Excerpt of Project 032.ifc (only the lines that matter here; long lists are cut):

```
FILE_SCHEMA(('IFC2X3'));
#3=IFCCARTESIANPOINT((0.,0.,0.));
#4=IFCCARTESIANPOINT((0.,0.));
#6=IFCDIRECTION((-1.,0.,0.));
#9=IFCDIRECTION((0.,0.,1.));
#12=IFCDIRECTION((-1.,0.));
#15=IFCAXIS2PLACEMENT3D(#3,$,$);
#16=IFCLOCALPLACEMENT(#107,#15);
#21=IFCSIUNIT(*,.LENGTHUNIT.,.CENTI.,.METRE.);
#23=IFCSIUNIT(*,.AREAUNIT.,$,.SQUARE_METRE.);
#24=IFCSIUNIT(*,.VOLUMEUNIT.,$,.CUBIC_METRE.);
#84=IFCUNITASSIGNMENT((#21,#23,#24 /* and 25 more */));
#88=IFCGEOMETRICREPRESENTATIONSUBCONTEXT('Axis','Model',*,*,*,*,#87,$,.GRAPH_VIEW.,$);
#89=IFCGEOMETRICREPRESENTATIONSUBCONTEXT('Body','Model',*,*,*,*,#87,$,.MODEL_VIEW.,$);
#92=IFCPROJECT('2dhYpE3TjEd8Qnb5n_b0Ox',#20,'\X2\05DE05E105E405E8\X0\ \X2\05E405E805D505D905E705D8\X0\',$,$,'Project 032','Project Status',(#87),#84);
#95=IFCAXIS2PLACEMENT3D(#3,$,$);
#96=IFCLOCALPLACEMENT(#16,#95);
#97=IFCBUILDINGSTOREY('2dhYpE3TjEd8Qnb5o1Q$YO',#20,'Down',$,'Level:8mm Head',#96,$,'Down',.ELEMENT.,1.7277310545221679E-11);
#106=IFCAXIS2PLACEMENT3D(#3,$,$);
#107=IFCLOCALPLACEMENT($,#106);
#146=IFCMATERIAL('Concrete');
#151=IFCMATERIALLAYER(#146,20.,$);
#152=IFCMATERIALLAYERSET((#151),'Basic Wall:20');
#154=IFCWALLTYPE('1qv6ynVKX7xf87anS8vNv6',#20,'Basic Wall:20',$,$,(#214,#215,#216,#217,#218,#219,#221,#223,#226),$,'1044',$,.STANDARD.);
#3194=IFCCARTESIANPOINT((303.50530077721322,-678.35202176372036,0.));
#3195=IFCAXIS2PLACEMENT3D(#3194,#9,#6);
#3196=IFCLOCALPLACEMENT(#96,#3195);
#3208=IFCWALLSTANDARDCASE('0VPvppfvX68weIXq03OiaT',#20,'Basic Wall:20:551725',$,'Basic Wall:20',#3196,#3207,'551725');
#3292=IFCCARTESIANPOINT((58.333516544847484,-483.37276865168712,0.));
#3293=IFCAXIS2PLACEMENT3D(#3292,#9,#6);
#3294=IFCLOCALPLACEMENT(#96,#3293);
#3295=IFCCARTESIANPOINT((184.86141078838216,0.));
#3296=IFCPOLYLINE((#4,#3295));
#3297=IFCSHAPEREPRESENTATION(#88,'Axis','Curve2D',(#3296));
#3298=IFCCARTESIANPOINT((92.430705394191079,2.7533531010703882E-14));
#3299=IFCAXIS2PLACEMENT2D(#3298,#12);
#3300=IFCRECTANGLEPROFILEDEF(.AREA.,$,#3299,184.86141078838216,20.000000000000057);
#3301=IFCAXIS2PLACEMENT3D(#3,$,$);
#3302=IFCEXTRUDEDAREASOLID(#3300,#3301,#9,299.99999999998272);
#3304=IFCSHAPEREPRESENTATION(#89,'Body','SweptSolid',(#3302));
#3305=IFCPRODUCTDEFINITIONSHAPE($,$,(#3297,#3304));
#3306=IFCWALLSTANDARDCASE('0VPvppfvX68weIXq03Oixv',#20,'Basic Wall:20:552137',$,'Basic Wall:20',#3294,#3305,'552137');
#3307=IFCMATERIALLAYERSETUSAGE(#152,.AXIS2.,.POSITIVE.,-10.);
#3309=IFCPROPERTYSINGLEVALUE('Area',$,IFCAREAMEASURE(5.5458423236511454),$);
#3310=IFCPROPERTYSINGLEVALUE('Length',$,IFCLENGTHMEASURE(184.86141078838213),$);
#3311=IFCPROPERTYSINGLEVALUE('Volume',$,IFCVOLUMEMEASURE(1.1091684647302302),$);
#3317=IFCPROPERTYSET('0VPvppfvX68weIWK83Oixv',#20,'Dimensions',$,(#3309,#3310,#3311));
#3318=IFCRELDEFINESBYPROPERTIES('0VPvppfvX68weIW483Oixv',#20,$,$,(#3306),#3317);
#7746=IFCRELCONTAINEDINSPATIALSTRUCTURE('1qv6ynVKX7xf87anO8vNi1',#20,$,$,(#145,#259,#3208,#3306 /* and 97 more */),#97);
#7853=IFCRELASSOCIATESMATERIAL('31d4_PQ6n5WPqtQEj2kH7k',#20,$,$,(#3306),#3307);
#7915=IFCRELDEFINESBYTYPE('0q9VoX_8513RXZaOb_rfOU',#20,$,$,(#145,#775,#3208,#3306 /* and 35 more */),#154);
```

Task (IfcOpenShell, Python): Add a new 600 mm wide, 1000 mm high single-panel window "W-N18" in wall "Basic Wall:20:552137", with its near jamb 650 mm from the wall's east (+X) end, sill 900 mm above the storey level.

```python
import numpy as np
import ifcopenshell
import ifcopenshell.api.feature
import ifcopenshell.api.geometry
import ifcopenshell.api.pset
import ifcopenshell.api.root
import ifcopenshell.api.spatial
import ifcopenshell.api.type
import ifcopenshell.geom
import ifcopenshell.util.element
import ifcopenshell.util.placement
import ifcopenshell.util.representation
import ifcopenshell.util.shape
import ifcopenshell.util.unit

model = ifcopenshell.open("Project 032.ifc")
unit_scale = ifcopenshell.util.unit.calculate_unit_scale(model)
area_scale = ifcopenshell.util.unit.calculate_unit_scale(model, "AREAUNIT")
volume_scale = ifcopenshell.util.unit.calculate_unit_scale(model, "VOLUMEUNIT")
settings = ifcopenshell.geom.settings()


def volume(element):
    """Net volume in cubic metres, openings subtracted."""
    shape = ifcopenshell.geom.create_shape(settings, element)
    return ifcopenshell.util.shape.get_volume(shape.geometry)


wall = model.by_guid("0VPvppfvX68weIXq03Oixv")
storey = ifcopenshell.util.element.get_container(wall, ifc_class="IfcBuildingStorey")
context = ifcopenshell.util.representation.get_context(model, "Model", "Body", "MODEL_VIEW")
before = volume(wall)

width, height, from_end, sill = 0.6, 1, 0.65, 0.9  # metres

# The wall runs along its own X axis, and the end named is its -X end.
wall_shape = ifcopenshell.geom.create_shape(settings, wall)
x, y, z = ifcopenshell.util.shape.get_vertices(wall_shape.geometry).T
start = x.min() + from_end
face, thickness = float(y.min()), float(y.max() - y.min())
wall_matrix = ifcopenshell.util.placement.get_local_placement(wall.ObjectPlacement)
level = ifcopenshell.util.placement.get_local_placement(storey.ObjectPlacement)[2, 3]


def in_wall(x, y):
    """Placement at x, y metres in the wall's axes, at sill height."""
    matrix = wall_matrix.copy()
    matrix[:, 3] = wall_matrix @ np.array([x / unit_scale, y / unit_scale, 0.0, 1.0])
    matrix[2, 3] = level + sill / unit_scale
    return matrix


# Opening: a box that overshoots both wall faces by 50 mm.
opening = ifcopenshell.api.root.create_entity(model, ifc_class="IfcOpeningElement")
box = ifcopenshell.api.geometry.add_wall_representation(
    model, context=context, length=width, height=height, thickness=thickness + 0.1
)
ifcopenshell.api.geometry.assign_representation(model, product=opening, representation=box)
ifcopenshell.api.geometry.edit_object_placement(model, product=opening, matrix=in_wall(start, face - 0.05), is_si=False)
ifcopenshell.api.feature.add_feature(model, feature=opening, element=wall)

window = ifcopenshell.api.root.create_entity(model, ifc_class="IfcWindow", name="W-N18")
window.OverallWidth, window.OverallHeight = width / unit_scale, height / unit_scale
body = ifcopenshell.api.geometry.add_window_representation(
    model,
    context=context,
    overall_width=window.OverallWidth,
    overall_height=window.OverallHeight,
    partition_type="SINGLE_PANEL",
)
ifcopenshell.api.geometry.assign_representation(model, product=window, representation=body)
ifcopenshell.api.spatial.assign_container(model, products=[window], relating_structure=storey)
fills = ifcopenshell.api.feature.add_filling(model, opening=opening, element=window)
fills.OwnerHistory = window.OwnerHistory  # required in IFC2X3

# IFC2X3 keeps the operation on the window style.
style = ifcopenshell.api.root.create_entity(model, ifc_class="IfcWindowStyle", name="W-N18")
style.OperationType, style.ConstructionType = "SINGLE_PANEL", "NOTDEFINED"
style.ParameterTakesPrecedence = style.Sizeable = False
ifcopenshell.api.type.assign_type(model, related_objects=[window], relating_type=style)

# Centre the window in the wall's thickness.
ifcopenshell.api.geometry.edit_object_placement(model, product=window, matrix=in_wall(start, face), is_si=False)
window_shape = ifcopenshell.geom.create_shape(settings, window)
depth = ifcopenshell.util.shape.get_vertices(window_shape.geometry)[:, 1]
offset = face + thickness / 2 - (depth.min() + depth.max()) / 2
ifcopenshell.api.geometry.edit_object_placement(model, product=window, matrix=in_wall(start, offset), is_si=False)

after = volume(wall)

# Update the wall's stored quantities.
pset = model.by_id(ifcopenshell.util.element.get_pset(wall, "Dimensions", should_inherit=False)["id"])
ifcopenshell.api.pset.edit_pset(model, pset=pset, properties={
    "Area": model.create_entity("IfcAreaMeasure", after / thickness / area_scale),
    "Volume": model.create_entity("IfcVolumeMeasure", after / volume_scale),
})

print(f"wall volume {before:.3f} -> {after:.3f} m3")

model.write("Project 032_rev.ifc")
```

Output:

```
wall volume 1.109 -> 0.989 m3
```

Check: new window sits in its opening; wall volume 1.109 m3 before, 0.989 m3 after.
